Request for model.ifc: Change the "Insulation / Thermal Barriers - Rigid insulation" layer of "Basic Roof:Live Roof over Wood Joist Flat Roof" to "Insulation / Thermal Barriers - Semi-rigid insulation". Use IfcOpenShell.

First a look at what the model holds.

```python
import ifcopenshell
import ifcopenshell.util.element

model = ifcopenshell.open("model.ifc")
print(model.schema)
for layer_set in model.by_type("IfcMaterialLayerSet"):
    if layer_set.LayerSetName == "Basic Roof:Live Roof over Wood Joist Flat Roof":
        for layer in layer_set.MaterialLayers:
            print(layer.id(), layer.Material and layer.Material.Name, layer.LayerThickness, sep=" | ")
        print(len(ifcopenshell.util.element.get_elements_by_material(model, layer_set)), "elements and types use it")
print(sorted(m.Name for m in model.by_type("IfcMaterial") if m.Name)[:60])
```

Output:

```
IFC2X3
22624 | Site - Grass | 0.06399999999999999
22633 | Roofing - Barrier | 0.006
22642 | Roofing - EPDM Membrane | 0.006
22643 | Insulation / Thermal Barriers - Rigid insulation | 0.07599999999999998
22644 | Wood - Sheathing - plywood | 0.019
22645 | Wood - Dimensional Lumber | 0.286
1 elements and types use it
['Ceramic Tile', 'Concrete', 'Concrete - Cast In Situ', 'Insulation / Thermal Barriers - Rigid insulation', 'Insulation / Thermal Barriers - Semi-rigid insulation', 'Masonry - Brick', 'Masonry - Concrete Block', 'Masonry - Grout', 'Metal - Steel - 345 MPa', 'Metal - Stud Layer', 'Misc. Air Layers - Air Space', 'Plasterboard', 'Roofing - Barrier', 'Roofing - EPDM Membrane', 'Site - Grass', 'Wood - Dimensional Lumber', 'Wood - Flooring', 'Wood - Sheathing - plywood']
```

```python
import ifcopenshell
import ifcopenshell.api.material

model = ifcopenshell.open("model.ifc")

layer_set = next(s for s in model.by_type("IfcMaterialLayerSet") if s.LayerSetName == "Basic Roof:Live Roof over Wood Joist Flat Roof")
layer = next(l for l in layer_set.MaterialLayers if l.Material and l.Material.Name == "Insulation / Thermal Barriers - Rigid insulation")
material = next(m for m in model.by_type("IfcMaterial") if m.Name == "Insulation / Thermal Barriers - Semi-rigid insulation")

# Point this one layer at the other material; renaming the old one would change it everywhere.
ifcopenshell.api.material.edit_layer(model, layer=layer, attributes={}, material=material)

print([l.Material.Name if l.Material else None for l in layer_set.MaterialLayers])

model.write("model_edited.ifc")
```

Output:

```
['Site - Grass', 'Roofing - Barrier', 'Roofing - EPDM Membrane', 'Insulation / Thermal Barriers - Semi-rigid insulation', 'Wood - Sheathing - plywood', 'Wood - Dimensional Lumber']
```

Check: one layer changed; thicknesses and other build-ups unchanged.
